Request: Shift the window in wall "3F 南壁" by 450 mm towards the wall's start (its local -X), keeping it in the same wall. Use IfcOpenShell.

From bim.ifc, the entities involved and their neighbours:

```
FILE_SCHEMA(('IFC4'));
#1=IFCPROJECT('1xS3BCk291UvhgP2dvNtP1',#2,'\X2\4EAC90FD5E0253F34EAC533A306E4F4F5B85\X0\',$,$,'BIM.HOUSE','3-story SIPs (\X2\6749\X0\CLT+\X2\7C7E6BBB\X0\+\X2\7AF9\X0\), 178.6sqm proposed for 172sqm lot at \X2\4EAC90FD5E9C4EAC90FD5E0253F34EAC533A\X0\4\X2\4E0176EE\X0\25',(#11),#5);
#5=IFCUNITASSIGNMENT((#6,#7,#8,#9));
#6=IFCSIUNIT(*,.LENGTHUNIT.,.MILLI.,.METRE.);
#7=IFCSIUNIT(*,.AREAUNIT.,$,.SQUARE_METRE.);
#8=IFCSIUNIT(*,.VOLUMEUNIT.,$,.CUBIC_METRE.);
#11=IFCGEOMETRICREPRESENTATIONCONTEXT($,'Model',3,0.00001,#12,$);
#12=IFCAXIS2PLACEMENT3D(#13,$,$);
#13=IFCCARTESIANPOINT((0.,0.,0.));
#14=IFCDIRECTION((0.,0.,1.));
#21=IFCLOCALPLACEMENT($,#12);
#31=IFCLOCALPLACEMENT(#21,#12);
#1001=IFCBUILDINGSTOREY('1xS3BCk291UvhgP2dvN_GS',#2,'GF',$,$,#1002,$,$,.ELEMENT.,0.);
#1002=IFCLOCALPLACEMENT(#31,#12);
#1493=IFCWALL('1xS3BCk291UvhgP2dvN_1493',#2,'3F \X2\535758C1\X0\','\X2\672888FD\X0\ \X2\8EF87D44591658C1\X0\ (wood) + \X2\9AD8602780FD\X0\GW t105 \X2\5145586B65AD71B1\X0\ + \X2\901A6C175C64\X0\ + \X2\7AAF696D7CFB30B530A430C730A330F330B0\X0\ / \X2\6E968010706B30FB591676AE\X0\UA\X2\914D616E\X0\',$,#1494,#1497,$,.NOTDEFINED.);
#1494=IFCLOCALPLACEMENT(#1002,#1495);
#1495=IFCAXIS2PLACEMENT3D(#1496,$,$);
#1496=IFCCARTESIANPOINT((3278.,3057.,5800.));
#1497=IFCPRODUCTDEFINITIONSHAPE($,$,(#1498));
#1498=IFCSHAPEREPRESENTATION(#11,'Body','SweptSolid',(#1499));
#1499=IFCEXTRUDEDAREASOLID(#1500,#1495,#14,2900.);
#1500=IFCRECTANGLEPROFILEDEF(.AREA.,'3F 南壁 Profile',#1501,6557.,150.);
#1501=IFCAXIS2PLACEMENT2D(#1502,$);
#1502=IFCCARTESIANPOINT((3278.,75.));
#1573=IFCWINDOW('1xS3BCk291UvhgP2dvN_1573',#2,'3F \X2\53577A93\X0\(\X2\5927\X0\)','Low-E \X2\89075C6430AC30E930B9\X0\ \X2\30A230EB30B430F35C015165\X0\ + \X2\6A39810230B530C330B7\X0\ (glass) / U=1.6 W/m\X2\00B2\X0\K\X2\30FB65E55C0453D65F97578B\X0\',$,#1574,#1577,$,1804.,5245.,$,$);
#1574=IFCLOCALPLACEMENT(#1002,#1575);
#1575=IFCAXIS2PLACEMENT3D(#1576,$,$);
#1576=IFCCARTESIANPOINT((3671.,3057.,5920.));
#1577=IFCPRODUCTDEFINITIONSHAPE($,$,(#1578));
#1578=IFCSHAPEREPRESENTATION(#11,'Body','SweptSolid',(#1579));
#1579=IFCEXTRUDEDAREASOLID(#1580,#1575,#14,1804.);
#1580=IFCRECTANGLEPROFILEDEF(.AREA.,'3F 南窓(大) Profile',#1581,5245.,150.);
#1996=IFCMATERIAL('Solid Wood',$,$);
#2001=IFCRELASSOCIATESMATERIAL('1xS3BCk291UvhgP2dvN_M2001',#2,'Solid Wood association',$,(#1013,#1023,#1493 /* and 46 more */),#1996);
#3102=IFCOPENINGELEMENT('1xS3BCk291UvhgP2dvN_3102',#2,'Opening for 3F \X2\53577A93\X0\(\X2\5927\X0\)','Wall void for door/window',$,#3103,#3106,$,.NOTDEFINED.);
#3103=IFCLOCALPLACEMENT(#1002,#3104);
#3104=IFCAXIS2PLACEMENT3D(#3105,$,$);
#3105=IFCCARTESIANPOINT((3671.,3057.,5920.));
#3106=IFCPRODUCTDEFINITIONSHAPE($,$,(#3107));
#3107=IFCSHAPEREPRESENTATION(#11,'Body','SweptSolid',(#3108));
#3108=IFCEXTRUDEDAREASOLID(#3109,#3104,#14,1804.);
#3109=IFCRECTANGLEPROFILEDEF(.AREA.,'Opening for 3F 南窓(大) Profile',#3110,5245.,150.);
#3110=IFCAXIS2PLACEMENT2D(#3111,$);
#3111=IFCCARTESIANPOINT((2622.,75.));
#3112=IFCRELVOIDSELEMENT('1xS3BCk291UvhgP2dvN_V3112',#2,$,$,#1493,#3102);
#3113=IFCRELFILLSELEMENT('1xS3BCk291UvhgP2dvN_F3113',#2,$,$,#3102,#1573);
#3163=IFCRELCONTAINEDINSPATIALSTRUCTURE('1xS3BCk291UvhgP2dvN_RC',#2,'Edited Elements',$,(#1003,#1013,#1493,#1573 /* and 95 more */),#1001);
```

```python
import ifcopenshell
import ifcopenshell.api.geometry
import ifcopenshell.util.placement

model = ifcopenshell.open("bim.ifc")

window = model.by_guid("1xS3BCk291UvhgP2dvN_1573")
opening = window.FillsVoids[0].RelatingOpeningElement
wall = opening.VoidsElements[0].RelatingBuildingElement

wall_matrix = ifcopenshell.util.placement.get_local_placement(wall.ObjectPlacement)
shift = wall_matrix[:3, 0] * -450.0
before = ifcopenshell.util.placement.get_local_placement(window.ObjectPlacement)[:3, 3].copy()

# The window is not placed relative to its opening, so move both.
for product in (opening, window):
    matrix = ifcopenshell.util.placement.get_local_placement(product.ObjectPlacement)
    matrix[:3, 3] += shift
    ifcopenshell.api.geometry.edit_object_placement(model, product=product, matrix=matrix, is_si=False)

after = ifcopenshell.util.placement.get_local_placement(window.ObjectPlacement)[:3, 3]
print("window moved by", (after - before).round(3) + 0.0)

model.write("bim_updated.ifc")
```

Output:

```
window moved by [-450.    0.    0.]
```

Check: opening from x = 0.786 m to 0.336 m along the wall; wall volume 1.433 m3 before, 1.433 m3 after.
